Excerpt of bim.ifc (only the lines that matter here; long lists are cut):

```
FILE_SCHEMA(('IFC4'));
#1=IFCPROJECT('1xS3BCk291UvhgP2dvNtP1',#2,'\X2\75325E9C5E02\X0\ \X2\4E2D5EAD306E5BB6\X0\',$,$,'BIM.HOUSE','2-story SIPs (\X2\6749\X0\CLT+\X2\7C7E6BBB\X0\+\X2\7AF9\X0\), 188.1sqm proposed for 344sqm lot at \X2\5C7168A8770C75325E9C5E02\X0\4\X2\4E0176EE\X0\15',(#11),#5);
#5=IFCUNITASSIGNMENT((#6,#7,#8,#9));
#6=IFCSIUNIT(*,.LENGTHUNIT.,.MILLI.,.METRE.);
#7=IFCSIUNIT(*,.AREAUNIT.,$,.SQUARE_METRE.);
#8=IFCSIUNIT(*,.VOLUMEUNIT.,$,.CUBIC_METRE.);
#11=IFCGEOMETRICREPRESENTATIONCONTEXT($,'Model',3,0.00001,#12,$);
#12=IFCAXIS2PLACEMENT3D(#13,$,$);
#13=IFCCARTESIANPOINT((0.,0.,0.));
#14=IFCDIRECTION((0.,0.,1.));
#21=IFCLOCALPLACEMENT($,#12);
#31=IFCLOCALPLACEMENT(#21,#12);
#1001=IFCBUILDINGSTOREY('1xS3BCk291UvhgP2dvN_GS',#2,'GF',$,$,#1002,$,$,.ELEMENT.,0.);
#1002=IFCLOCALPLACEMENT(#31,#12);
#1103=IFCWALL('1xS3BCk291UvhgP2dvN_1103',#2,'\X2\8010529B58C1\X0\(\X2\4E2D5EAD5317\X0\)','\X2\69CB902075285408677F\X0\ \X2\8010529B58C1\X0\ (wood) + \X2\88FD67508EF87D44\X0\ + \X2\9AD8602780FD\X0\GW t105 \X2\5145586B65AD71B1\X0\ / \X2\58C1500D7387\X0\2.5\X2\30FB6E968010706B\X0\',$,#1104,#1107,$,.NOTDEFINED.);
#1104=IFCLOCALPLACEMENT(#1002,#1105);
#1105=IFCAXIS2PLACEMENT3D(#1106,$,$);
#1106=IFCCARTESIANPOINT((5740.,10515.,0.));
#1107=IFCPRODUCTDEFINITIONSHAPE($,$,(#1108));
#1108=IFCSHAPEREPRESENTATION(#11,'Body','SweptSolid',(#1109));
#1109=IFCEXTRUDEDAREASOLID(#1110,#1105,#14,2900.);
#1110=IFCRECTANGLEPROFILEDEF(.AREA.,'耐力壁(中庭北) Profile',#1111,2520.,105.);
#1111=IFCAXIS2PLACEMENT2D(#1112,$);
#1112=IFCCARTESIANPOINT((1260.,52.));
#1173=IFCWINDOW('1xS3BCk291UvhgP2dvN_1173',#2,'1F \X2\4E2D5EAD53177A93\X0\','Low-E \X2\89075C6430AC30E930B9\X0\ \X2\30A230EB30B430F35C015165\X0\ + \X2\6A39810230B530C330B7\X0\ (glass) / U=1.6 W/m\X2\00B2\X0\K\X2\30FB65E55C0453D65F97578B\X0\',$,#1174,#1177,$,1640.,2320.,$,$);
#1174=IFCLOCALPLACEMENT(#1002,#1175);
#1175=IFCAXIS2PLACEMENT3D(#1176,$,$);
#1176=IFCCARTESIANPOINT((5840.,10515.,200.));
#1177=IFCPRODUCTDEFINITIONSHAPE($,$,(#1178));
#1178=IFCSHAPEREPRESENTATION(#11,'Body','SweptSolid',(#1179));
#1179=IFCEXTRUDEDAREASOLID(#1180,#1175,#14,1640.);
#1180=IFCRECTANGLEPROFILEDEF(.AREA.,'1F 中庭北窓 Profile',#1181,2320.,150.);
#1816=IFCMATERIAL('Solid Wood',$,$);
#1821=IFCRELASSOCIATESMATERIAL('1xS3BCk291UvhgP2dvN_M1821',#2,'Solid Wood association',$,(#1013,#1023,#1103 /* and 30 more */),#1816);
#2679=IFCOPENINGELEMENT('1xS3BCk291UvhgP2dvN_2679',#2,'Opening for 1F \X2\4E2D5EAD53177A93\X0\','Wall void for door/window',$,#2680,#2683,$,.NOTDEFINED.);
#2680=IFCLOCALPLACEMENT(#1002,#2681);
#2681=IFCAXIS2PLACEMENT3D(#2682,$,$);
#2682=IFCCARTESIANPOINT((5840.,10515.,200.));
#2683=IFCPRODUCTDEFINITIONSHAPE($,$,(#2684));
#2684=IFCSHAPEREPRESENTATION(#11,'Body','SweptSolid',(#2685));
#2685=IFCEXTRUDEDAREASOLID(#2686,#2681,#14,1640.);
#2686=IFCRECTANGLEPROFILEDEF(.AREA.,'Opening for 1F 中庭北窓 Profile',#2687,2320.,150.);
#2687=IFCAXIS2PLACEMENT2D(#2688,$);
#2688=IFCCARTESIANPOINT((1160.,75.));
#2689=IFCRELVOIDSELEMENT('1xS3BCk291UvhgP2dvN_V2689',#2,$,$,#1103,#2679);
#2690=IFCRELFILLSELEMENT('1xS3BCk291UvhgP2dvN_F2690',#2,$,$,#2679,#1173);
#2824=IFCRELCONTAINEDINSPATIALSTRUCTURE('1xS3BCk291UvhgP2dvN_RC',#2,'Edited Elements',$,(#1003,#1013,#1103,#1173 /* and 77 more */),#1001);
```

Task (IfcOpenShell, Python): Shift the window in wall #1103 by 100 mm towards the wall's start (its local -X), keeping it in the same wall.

```python
import ifcopenshell
import ifcopenshell.api.geometry
import ifcopenshell.util.placement

model = ifcopenshell.open("bim.ifc")

window = model.by_guid("1xS3BCk291UvhgP2dvN_1173")
opening = window.FillsVoids[0].RelatingOpeningElement
wall = opening.VoidsElements[0].RelatingBuildingElement

wall_matrix = ifcopenshell.util.placement.get_local_placement(wall.ObjectPlacement)
shift = wall_matrix[:3, 0] * -100.0
before = ifcopenshell.util.placement.get_local_placement(window.ObjectPlacement)[:3, 3].copy()

# The window is not placed relative to its opening, so move both.
for product in (opening, window):
    matrix = ifcopenshell.util.placement.get_local_placement(product.ObjectPlacement)
    matrix[:3, 3] += shift
    ifcopenshell.api.geometry.edit_object_placement(model, product=product, matrix=matrix, is_si=False)

after = ifcopenshell.util.placement.get_local_placement(window.ObjectPlacement)[:3, 3]
print("window moved by", (after - before).round(3) + 0.0)

model.write("bim_v2.ifc")
```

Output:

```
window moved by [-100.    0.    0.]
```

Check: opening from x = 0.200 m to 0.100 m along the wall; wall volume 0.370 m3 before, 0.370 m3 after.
